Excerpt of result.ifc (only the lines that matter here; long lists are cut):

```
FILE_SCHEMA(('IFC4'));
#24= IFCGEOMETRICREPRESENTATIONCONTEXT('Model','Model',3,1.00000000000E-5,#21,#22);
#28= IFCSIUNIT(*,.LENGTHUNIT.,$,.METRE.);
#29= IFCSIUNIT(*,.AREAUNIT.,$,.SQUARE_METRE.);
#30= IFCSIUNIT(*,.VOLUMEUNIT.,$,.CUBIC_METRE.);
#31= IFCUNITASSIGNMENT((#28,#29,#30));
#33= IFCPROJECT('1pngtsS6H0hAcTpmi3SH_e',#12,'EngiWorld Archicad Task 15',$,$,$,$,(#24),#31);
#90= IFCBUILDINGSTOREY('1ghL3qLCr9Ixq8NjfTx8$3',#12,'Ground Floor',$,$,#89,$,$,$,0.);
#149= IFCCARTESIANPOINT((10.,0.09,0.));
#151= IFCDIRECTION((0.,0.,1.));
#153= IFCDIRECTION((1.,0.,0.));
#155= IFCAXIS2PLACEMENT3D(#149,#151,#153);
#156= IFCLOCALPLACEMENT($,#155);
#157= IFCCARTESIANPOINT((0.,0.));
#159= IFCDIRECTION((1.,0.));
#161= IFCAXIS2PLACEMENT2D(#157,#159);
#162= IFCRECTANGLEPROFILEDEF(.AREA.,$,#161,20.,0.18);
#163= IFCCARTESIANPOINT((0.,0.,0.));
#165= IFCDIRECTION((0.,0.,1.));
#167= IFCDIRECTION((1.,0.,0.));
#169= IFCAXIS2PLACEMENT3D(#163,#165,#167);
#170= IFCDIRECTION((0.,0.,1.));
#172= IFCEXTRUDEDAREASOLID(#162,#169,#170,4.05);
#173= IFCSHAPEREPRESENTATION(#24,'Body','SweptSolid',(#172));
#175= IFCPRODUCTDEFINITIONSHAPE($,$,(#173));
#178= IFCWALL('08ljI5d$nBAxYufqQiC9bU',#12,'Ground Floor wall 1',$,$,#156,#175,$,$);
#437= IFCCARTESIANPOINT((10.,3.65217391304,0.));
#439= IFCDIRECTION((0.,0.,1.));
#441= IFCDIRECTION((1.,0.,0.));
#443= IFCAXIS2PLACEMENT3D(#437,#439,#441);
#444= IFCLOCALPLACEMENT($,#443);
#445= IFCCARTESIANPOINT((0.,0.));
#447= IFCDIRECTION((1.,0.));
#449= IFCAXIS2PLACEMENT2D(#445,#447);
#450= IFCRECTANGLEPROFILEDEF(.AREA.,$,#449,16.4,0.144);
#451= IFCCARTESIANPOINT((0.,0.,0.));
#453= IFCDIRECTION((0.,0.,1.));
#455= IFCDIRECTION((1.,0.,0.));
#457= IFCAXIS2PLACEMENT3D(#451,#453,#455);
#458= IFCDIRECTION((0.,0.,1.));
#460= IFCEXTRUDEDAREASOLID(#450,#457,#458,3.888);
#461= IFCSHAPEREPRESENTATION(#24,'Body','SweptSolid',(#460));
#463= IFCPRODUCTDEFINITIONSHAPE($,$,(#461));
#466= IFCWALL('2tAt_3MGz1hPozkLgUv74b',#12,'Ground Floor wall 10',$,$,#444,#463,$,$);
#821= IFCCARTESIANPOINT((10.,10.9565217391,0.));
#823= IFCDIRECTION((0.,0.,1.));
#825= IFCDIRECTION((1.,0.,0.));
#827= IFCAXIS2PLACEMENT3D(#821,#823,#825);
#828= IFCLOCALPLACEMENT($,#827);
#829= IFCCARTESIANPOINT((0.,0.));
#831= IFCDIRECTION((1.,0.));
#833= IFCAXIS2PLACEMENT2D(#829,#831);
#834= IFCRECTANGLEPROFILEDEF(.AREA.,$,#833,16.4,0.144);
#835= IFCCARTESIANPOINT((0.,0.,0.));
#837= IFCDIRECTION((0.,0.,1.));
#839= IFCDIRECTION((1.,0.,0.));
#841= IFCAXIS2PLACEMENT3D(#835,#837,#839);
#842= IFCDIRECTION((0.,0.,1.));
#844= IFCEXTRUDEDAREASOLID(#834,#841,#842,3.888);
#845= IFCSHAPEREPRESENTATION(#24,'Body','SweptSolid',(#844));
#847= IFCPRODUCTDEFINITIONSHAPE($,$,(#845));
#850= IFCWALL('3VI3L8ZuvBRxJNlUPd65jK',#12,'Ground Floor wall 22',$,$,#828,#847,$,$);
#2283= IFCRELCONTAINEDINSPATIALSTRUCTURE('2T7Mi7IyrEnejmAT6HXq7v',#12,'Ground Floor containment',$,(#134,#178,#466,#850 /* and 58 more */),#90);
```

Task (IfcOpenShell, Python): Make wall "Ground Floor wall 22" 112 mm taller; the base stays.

```python
import ifcopenshell
import ifcopenshell.geom
import ifcopenshell.util.shape

model = ifcopenshell.open("result.ifc")
settings = ifcopenshell.geom.settings()


def volume(element):
    """Net volume in cubic metres, openings subtracted."""
    shape = ifcopenshell.geom.create_shape(settings, element)
    return ifcopenshell.util.shape.get_volume(shape.geometry)


wall = model.by_guid("3VI3L8ZuvBRxJNlUPd65jK")
before = volume(wall)

body = next(r for r in wall.Representation.Representations if r.RepresentationIdentifier == "Body")
solid = body.Items[0]
old_height = solid.Depth
solid.Depth += 0.112
after = volume(wall)

print(f"height {old_height:g} -> {solid.Depth:g}, volume {before:.3f} -> {after:.3f} m3")

model.write("result_edited.ifc")
```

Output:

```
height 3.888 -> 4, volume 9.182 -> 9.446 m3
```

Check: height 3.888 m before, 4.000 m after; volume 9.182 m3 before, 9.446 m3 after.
